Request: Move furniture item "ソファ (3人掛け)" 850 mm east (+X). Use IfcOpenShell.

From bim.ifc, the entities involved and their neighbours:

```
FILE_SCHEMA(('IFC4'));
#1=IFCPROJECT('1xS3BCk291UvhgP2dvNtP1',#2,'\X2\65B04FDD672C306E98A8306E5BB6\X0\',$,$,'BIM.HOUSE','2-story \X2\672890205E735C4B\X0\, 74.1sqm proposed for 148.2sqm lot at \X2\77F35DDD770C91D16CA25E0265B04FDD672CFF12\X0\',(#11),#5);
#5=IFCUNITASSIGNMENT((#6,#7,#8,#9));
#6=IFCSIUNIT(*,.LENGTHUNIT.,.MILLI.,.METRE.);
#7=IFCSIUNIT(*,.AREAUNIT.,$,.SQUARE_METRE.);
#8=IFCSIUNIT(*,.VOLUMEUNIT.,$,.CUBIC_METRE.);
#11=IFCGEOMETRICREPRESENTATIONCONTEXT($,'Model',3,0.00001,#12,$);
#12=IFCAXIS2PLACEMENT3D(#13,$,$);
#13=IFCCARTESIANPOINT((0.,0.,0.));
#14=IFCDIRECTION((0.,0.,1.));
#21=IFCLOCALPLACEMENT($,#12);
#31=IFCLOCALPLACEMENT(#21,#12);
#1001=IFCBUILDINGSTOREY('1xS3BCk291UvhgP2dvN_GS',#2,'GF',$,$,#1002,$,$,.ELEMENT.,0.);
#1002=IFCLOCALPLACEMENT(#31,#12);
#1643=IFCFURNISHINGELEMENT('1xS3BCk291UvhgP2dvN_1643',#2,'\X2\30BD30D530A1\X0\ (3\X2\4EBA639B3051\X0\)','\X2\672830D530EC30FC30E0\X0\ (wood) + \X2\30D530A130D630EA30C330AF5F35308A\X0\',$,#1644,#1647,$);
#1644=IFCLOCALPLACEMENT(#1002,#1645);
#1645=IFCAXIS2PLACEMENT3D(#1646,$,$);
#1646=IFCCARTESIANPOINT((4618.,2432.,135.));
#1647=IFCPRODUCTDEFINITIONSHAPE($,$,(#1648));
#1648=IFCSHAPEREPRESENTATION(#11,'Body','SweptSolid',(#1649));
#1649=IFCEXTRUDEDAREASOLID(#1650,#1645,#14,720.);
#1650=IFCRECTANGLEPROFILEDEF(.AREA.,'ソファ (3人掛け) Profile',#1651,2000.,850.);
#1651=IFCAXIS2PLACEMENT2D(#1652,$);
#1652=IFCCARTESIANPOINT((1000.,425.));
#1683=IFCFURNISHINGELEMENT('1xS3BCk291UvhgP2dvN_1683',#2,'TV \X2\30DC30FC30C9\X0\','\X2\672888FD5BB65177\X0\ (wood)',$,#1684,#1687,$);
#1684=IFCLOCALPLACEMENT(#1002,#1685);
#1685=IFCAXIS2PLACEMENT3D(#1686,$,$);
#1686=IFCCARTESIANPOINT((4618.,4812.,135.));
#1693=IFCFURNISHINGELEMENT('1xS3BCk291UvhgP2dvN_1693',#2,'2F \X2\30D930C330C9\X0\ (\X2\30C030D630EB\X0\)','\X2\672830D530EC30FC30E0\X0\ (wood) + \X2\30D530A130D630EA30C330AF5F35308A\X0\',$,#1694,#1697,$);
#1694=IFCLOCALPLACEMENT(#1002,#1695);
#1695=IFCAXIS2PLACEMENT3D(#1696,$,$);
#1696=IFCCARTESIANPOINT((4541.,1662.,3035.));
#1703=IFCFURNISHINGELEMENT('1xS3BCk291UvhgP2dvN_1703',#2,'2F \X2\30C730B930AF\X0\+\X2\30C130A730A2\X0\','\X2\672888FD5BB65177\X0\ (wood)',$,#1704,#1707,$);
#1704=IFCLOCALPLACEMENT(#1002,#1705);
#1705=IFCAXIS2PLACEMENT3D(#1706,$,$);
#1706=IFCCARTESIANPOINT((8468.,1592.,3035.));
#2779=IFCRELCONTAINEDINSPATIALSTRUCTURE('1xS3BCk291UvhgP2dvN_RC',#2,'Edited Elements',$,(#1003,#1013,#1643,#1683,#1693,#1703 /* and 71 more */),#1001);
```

```python
import ifcopenshell
import ifcopenshell.api.geometry
import ifcopenshell.util.placement
import ifcopenshell.util.unit

model = ifcopenshell.open("bim.ifc")
unit_scale = ifcopenshell.util.unit.calculate_unit_scale(model)

item = model.by_id(1643)
matrix = ifcopenshell.util.placement.get_local_placement(item.ObjectPlacement)
matrix[0, 3] += 0.85 / unit_scale
ifcopenshell.api.geometry.edit_object_placement(model, product=item, matrix=matrix, is_si=False)

print(ifcopenshell.util.placement.get_local_placement(item.ObjectPlacement).round(3) + 0.0)

model.write("bim_v2.ifc")
```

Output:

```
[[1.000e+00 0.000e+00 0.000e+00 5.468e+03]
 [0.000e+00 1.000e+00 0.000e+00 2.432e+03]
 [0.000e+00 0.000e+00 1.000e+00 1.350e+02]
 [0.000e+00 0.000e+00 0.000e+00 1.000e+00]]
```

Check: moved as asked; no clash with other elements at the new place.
